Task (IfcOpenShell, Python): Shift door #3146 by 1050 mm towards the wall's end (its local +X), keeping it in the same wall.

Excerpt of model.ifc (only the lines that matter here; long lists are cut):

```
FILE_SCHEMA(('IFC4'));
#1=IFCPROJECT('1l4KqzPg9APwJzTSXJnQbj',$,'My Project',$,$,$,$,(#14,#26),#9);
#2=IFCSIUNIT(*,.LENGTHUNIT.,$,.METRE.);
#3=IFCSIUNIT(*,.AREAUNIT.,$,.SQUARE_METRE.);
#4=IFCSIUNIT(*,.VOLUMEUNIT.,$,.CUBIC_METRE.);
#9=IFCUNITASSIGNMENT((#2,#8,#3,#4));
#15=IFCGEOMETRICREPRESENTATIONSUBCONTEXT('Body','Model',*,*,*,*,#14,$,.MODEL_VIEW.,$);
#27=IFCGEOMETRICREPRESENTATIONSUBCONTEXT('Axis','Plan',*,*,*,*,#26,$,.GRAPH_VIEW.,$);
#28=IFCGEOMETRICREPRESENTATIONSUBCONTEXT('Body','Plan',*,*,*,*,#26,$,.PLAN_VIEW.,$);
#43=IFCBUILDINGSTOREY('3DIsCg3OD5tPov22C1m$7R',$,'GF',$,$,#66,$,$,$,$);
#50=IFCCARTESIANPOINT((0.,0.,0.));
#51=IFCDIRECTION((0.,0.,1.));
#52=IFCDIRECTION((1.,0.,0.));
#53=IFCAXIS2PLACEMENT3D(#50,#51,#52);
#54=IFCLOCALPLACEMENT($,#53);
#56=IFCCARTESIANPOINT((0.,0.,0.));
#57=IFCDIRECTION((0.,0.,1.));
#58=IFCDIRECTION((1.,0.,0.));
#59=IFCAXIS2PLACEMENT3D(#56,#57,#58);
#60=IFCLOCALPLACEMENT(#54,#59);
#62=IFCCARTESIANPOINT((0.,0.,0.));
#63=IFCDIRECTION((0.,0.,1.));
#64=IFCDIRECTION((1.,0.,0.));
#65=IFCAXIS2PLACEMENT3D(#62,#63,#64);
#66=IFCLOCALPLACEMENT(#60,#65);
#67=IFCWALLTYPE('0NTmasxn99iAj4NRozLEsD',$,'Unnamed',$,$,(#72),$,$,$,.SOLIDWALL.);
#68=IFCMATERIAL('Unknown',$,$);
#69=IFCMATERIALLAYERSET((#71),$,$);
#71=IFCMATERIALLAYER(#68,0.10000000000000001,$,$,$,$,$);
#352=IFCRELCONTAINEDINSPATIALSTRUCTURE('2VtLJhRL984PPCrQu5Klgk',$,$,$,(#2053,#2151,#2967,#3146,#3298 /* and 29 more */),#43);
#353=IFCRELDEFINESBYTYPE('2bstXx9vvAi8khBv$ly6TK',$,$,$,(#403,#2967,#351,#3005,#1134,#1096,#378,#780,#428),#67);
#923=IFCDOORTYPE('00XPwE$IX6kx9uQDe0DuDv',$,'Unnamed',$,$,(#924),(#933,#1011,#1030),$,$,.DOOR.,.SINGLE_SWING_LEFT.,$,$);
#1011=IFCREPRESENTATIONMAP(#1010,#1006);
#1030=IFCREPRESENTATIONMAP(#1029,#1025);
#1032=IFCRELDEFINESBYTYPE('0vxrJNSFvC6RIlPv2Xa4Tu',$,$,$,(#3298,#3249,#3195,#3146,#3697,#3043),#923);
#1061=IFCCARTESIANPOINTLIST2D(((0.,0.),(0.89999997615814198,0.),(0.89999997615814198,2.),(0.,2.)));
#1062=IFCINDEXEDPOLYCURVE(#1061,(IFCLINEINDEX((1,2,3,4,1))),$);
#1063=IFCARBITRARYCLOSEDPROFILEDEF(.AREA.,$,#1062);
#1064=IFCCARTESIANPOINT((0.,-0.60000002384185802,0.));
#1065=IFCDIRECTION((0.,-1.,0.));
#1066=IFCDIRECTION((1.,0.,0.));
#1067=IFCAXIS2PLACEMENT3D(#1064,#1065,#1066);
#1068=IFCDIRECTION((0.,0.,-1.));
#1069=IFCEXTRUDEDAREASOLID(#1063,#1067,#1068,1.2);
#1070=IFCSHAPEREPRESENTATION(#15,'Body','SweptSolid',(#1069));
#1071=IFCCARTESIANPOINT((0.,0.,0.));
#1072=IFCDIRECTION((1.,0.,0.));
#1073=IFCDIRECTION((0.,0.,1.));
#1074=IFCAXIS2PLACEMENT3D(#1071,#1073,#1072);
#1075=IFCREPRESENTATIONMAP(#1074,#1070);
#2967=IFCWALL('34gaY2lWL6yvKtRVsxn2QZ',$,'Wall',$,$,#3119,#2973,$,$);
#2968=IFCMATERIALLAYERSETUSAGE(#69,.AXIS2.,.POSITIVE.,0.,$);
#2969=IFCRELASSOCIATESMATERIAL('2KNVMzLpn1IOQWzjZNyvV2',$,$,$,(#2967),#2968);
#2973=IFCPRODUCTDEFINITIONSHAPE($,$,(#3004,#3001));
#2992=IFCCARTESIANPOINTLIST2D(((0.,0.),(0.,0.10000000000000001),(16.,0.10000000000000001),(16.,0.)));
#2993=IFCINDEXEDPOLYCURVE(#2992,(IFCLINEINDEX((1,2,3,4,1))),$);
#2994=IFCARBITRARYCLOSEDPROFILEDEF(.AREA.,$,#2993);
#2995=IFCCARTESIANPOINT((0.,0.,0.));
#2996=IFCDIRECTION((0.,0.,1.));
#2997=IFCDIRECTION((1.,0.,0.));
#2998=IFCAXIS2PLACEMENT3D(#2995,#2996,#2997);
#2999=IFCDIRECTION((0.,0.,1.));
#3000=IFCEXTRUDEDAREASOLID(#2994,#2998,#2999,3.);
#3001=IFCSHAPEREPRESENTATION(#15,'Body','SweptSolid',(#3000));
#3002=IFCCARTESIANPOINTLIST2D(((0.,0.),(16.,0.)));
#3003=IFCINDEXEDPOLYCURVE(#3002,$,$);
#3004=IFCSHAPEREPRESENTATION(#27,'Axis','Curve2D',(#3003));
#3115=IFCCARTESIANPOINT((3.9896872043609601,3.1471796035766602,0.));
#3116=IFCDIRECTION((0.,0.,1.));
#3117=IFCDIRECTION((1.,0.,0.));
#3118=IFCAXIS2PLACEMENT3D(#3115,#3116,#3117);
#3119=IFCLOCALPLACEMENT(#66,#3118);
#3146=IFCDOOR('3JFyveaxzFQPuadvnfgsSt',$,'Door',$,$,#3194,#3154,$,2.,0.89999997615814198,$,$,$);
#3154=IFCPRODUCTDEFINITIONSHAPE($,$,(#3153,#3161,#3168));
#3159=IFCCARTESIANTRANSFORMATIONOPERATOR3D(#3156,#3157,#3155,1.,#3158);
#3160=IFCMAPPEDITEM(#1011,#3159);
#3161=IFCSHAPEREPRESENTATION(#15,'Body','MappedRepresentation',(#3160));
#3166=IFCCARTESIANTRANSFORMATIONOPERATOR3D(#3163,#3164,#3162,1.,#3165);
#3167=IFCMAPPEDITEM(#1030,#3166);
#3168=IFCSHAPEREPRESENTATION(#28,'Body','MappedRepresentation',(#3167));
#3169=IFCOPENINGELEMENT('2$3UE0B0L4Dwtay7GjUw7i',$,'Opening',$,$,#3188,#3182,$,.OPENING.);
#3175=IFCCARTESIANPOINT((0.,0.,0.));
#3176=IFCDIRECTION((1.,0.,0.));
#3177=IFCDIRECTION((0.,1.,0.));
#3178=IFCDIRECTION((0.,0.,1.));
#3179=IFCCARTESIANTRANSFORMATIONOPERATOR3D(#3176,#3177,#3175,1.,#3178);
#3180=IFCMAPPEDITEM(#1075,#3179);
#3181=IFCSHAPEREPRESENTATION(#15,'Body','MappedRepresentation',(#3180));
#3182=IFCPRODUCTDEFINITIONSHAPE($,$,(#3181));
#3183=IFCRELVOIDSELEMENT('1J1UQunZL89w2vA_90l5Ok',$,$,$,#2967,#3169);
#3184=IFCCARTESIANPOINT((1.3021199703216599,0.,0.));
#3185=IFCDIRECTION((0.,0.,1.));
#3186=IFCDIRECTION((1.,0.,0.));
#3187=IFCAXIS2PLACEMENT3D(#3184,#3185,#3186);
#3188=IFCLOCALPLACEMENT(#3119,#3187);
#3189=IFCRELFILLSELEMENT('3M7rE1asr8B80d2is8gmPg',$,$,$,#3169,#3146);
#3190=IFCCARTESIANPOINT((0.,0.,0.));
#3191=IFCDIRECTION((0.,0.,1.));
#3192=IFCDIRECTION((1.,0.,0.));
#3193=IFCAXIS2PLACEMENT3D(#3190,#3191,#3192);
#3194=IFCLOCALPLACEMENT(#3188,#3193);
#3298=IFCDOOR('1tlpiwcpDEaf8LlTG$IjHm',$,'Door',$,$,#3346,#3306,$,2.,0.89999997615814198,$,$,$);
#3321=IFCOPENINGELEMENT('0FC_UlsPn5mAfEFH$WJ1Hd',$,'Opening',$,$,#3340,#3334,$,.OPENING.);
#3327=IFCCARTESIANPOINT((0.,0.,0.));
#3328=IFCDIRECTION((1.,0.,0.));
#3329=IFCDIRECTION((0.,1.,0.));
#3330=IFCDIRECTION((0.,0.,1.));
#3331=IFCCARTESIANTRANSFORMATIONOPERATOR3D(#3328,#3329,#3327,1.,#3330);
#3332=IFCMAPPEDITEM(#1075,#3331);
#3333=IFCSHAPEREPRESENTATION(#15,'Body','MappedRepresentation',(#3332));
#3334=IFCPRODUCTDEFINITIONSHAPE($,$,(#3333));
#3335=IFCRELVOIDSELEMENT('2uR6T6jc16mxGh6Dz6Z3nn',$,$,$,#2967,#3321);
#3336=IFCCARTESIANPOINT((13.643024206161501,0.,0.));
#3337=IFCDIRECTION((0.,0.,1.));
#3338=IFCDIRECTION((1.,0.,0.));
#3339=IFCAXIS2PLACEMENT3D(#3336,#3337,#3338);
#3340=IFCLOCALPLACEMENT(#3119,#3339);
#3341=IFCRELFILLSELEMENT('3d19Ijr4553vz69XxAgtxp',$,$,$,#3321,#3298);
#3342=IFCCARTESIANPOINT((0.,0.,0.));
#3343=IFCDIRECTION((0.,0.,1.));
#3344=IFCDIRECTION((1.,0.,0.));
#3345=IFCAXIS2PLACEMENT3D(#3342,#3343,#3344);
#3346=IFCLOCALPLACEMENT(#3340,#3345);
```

```python
import ifcopenshell
import ifcopenshell.api.geometry
import ifcopenshell.util.placement
import ifcopenshell.util.unit

model = ifcopenshell.open("model.ifc")
unit_scale = ifcopenshell.util.unit.calculate_unit_scale(model)

door = model.by_guid("3JFyveaxzFQPuadvnfgsSt")
opening = door.FillsVoids[0].RelatingOpeningElement
wall = opening.VoidsElements[0].RelatingBuildingElement

wall_matrix = ifcopenshell.util.placement.get_local_placement(wall.ObjectPlacement)
shift = wall_matrix[:3, 0] * 1.05 / unit_scale
before = ifcopenshell.util.placement.get_local_placement(door.ObjectPlacement)[:3, 3].copy()

# The door is placed relative to its opening, so it follows when the opening moves.
matrix = ifcopenshell.util.placement.get_local_placement(opening.ObjectPlacement)
matrix[:3, 3] += shift
ifcopenshell.api.geometry.edit_object_placement(
    model, product=opening, matrix=matrix, is_si=False, should_transform_children=True
)

after = ifcopenshell.util.placement.get_local_placement(door.ObjectPlacement)[:3, 3]
print("door moved by", (after - before).round(3) + 0.0)

model.write("model_rev.ifc")
```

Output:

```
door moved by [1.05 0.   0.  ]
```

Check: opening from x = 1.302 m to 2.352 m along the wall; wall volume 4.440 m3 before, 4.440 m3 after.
